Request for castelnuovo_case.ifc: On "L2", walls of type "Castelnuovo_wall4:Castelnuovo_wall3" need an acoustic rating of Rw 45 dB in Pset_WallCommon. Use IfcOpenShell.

First a look at what the model holds.

```python
import ifcopenshell
import ifcopenshell.util.element

model = ifcopenshell.open("castelnuovo_case.ifc")
print(model.schema)
storey = next(s for s in model.by_type("IfcBuildingStorey") if s.Name == "L2")
walls = [e for e in ifcopenshell.util.element.get_decomposition(storey) if e.is_a("IfcWall")]
seen = {}
for e in walls:
    element_type = ifcopenshell.util.element.get_type(e)
    key = (element_type.Name if element_type != e and element_type else None, ifcopenshell.util.element.get_pset(e, "Pset_WallCommon", "AcousticRating"))
    seen[key] = seen.get(key, 0) + 1
for (name, value), count in sorted(seen.items(), key=str):
    print(count, "x", name, "|", value)
```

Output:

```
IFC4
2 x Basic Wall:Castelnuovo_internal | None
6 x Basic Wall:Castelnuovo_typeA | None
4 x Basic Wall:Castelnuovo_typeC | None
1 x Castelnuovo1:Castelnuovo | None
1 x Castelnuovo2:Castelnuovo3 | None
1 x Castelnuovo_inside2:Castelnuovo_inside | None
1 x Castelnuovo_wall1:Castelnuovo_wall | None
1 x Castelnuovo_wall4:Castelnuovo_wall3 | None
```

```python
import ifcopenshell
import ifcopenshell.api.pset
import ifcopenshell.util.element

model = ifcopenshell.open("castelnuovo_case.ifc")

storey = next(s for s in model.by_type("IfcBuildingStorey") if s.Name == "L2")
walls = [e for e in ifcopenshell.util.element.get_decomposition(storey) if e.is_a("IfcWall")]

count = 0
for e in walls:
    element_type = ifcopenshell.util.element.get_type(e)
    if element_type in (None, e) or element_type.Name != "Castelnuovo_wall4:Castelnuovo_wall3":
        continue
    # add_pset returns the element's existing set when there is one.
    pset = ifcopenshell.api.pset.add_pset(model, product=e, name="Pset_WallCommon")
    ifcopenshell.api.pset.edit_pset(model, pset=pset, properties={"AcousticRating": "Rw 45 dB"})
    count += 1

print(count, "walls updated")

model.write("castelnuovo_case_v2.ifc")
```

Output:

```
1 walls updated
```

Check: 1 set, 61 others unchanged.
